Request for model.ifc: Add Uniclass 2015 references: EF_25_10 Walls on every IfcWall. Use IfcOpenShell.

First a look at what the model holds.

```python
import ifcopenshell

model = ifcopenshell.open("model.ifc")
print(model.schema)
print("classifications:", [c.Name for c in model.by_type("IfcClassification")])
for ifc_class in ("IfcDoor", "IfcRoof", "IfcStair", "IfcWall", "IfcWindow"):
    print(ifc_class, len(model.by_type(ifc_class)))
```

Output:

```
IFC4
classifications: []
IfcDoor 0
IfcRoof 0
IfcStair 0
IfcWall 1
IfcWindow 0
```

```python
import ifcopenshell
import ifcopenshell.api.classification

model = ifcopenshell.open("model.ifc")

system = ifcopenshell.api.classification.add_classification(model, classification="Uniclass 2015")

codes = {
    "IfcWall": ("EF_25_10", "Walls"),
}
for ifc_class, (code, name) in codes.items():
    products = model.by_type(ifc_class)
    ifcopenshell.api.classification.add_reference(
        model, products=products, classification=system, identification=code, name=name
    )
    print(code, len(products))

model.write("model_v2.ifc")
```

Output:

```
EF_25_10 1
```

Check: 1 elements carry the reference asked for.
